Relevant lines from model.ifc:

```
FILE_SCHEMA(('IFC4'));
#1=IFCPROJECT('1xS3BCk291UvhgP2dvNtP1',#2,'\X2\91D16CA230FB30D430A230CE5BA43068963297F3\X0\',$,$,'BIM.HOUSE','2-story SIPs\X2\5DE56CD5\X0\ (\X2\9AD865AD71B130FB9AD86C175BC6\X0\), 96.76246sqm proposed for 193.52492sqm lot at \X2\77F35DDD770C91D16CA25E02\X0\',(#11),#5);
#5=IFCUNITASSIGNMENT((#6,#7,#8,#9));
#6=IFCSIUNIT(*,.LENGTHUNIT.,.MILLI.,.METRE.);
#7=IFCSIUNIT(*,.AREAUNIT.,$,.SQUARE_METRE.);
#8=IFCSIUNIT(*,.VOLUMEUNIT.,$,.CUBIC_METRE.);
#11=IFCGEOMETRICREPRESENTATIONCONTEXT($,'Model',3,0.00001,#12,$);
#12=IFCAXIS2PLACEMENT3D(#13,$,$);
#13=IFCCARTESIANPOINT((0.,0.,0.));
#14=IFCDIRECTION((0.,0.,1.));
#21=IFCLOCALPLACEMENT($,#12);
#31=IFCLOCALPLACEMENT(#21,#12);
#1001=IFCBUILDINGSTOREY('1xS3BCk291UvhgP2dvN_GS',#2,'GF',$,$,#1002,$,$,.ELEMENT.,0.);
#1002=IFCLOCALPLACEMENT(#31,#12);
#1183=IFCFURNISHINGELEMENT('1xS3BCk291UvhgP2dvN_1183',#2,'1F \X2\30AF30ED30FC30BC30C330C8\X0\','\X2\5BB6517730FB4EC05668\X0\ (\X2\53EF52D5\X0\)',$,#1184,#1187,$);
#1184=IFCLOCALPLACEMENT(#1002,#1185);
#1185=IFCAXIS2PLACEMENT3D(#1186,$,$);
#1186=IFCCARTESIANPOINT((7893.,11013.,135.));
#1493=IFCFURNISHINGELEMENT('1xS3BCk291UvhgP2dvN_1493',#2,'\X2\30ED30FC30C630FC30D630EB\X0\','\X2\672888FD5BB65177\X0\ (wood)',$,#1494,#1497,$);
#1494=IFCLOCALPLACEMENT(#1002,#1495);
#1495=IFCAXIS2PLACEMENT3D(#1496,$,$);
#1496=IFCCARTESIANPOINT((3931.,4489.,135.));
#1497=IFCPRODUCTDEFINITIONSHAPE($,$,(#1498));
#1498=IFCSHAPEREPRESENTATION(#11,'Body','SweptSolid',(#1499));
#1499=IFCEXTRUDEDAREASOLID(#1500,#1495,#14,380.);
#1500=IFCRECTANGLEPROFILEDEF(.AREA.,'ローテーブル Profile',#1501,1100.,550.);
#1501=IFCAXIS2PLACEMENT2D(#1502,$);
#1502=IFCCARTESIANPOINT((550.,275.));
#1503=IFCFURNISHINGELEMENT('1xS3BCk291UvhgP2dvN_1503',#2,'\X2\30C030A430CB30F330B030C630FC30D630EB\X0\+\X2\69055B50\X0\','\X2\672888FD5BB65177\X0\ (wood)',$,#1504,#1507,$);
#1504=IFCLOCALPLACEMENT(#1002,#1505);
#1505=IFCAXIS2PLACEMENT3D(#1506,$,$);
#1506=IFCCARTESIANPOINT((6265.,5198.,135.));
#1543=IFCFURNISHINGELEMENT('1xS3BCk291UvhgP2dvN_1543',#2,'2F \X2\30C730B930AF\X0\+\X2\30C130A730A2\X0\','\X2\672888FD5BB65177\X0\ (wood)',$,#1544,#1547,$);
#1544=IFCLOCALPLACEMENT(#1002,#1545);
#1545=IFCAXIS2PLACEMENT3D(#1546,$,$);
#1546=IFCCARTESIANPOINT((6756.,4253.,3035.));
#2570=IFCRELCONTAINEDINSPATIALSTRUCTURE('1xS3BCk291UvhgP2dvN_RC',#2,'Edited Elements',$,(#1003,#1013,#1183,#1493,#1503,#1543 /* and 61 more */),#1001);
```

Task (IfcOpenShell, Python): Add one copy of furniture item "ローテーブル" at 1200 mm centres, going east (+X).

```python
import numpy as np
import ifcopenshell
import ifcopenshell.api.geometry
import ifcopenshell.api.root
import ifcopenshell.util.element
import ifcopenshell.util.placement
import ifcopenshell.util.unit

model = ifcopenshell.open("model.ifc")
unit_scale = ifcopenshell.util.unit.calculate_unit_scale(model)


def reuse_history(source, copy):
    """copy_class also copies each property set's owner history, people and application; keep the originals."""
    for rel in copy.IsDefinedBy:
        if rel.is_a("IfcRelDefinesByProperties") and (history := rel.RelatingPropertyDefinition.OwnerHistory):
            rel.RelatingPropertyDefinition.OwnerHistory = source.OwnerHistory
            ifcopenshell.util.element.remove_deep2(model, history)


source = model.by_guid("1xS3BCk291UvhgP2dvN_1493")
base = ifcopenshell.util.placement.get_local_placement(source.ObjectPlacement)
step = np.array([1.0, 0.0, 0.0]) * 1.2 / unit_scale

for i in range(1, 2):
    copy = ifcopenshell.api.root.copy_class(model, product=source)
    copy.Representation = ifcopenshell.util.element.copy_deep(
        model, source.Representation, exclude=["IfcGeometricRepresentationContext", "IfcRepresentationMap"]
    )
    reuse_history(source, copy)
    matrix = base.copy()
    matrix[:3, 3] += i * step
    print("added at", matrix[:3, 3].round(3) + 0.0)
    ifcopenshell.api.geometry.edit_object_placement(model, product=copy, matrix=matrix, is_si=False)

model.write("model_updated.ifc")
```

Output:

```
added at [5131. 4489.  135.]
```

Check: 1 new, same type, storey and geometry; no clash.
